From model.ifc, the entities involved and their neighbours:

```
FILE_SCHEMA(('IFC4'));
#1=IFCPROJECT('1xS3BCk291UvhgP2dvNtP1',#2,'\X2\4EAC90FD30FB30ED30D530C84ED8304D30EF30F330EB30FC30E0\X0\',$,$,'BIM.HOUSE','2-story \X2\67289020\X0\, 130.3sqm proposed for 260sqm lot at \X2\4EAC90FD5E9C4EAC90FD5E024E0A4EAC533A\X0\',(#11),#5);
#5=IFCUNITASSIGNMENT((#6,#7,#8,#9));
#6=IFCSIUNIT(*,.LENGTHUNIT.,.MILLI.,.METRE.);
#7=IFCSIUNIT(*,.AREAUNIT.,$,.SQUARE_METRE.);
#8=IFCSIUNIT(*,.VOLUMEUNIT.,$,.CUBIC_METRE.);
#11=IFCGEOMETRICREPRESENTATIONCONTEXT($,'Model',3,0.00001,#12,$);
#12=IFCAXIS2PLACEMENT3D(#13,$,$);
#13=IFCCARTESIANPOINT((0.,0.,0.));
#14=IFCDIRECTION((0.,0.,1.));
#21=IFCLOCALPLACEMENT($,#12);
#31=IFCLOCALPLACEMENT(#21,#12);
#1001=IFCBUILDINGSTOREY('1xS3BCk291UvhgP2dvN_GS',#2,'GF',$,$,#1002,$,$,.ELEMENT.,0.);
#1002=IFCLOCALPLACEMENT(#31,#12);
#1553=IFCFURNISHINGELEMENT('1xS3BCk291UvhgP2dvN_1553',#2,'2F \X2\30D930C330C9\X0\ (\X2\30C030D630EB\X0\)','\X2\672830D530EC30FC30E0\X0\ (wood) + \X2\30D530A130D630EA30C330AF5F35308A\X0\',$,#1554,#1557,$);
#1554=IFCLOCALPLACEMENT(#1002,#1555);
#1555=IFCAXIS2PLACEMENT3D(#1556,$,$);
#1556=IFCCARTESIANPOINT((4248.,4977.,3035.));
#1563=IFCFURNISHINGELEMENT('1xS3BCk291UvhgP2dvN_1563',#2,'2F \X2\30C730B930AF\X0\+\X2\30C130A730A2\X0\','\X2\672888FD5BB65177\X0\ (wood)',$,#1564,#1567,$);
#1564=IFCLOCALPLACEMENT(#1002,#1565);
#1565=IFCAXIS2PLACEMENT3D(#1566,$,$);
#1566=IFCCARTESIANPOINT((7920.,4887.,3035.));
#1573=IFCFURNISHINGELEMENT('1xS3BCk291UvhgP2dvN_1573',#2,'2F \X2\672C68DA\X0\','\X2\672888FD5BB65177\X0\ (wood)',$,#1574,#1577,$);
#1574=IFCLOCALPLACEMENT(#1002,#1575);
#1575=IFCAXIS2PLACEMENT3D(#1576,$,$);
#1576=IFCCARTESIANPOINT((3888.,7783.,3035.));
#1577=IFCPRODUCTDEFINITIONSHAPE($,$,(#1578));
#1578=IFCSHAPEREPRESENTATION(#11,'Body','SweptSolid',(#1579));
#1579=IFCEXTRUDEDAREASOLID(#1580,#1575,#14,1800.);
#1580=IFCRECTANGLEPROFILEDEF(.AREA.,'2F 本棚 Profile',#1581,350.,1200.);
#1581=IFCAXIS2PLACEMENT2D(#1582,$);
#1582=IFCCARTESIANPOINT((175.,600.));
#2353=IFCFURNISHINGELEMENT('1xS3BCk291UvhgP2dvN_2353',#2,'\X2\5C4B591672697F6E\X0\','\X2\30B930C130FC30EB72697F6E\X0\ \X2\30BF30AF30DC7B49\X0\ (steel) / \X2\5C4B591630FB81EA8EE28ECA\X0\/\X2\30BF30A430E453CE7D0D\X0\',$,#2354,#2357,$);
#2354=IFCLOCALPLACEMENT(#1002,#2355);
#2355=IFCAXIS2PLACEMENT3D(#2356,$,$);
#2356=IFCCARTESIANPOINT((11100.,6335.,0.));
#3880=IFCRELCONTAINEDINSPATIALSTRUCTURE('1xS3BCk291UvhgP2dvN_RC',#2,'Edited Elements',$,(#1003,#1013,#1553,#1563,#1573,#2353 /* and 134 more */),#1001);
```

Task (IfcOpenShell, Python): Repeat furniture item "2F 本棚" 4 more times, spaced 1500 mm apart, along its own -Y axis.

```python
import ifcopenshell
import ifcopenshell.api.geometry
import ifcopenshell.api.root
import ifcopenshell.util.element
import ifcopenshell.util.placement
import ifcopenshell.util.unit

model = ifcopenshell.open("model.ifc")
unit_scale = ifcopenshell.util.unit.calculate_unit_scale(model)


def reuse_history(source, copy):
    """copy_class also copies each property set's owner history, people and application; keep the originals."""
    for rel in copy.IsDefinedBy:
        if rel.is_a("IfcRelDefinesByProperties") and (history := rel.RelatingPropertyDefinition.OwnerHistory):
            rel.RelatingPropertyDefinition.OwnerHistory = source.OwnerHistory
            ifcopenshell.util.element.remove_deep2(model, history)


source = model.by_guid("1xS3BCk291UvhgP2dvN_1573")
base = ifcopenshell.util.placement.get_local_placement(source.ObjectPlacement)
step = -base[:3, 1] * 1.5 / unit_scale

for i in range(1, 5):
    copy = ifcopenshell.api.root.copy_class(model, product=source)
    copy.Representation = ifcopenshell.util.element.copy_deep(
        model, source.Representation, exclude=["IfcGeometricRepresentationContext", "IfcRepresentationMap"]
    )
    reuse_history(source, copy)
    matrix = base.copy()
    matrix[:3, 3] += i * step
    print("added at", matrix[:3, 3].round(3) + 0.0)
    ifcopenshell.api.geometry.edit_object_placement(model, product=copy, matrix=matrix, is_si=False)

model.write("model-out.ifc")
```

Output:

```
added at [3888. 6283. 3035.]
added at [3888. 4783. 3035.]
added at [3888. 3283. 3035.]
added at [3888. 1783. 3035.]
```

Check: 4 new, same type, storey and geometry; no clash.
